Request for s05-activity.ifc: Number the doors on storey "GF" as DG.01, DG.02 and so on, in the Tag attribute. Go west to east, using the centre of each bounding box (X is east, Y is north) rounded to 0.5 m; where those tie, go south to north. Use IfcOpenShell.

First a look at what the model holds.

```python
import ifcopenshell
import ifcopenshell.util.element
import ifcopenshell.util.placement

model = ifcopenshell.open("s05-activity.ifc")
print(model.schema)
storey = next(s for s in model.by_type("IfcBuildingStorey") if s.Name == "GF")
doors = [e for e in ifcopenshell.util.element.get_decomposition(storey) if e.is_a("IfcDoor")]
for e in sorted(doors, key=lambda e: e.id()):
    origin = ifcopenshell.util.placement.get_local_placement(e.ObjectPlacement)[:3, 3]
    print(e.id(), e.Tag, e.Name, origin.round(2) + 0.0, sep=" | ")
```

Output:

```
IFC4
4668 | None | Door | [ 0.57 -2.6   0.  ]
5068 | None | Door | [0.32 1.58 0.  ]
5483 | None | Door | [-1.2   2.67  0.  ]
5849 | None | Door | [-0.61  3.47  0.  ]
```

```python
import ifcopenshell
import ifcopenshell.geom
import ifcopenshell.util.element
import ifcopenshell.util.shape

model = ifcopenshell.open("s05-activity.ifc")
settings = ifcopenshell.geom.settings()
settings.set("use-world-coords", True)


def centre(element):
    shape = ifcopenshell.geom.create_shape(settings, element)
    return ifcopenshell.util.shape.get_bbox_centroid(shape.geometry)


storey = next(s for s in model.by_type("IfcBuildingStorey") if s.Name == "GF")
doors = [e for e in ifcopenshell.util.element.get_decomposition(storey) if e.is_a("IfcDoor")]

# Insertion points can sit at a corner or the storey origin, so sort by the geometry (in metres).
centres = {e: centre(e) for e in doors}
doors.sort(key=lambda e: (round(centres[e][0] / 0.5), centres[e][1]))

for i, e in enumerate(doors, start=1):
    number = f"DG.{i:02d}"
    e.Tag = number
    print(e.id(), number)

model.write("s05-activity_rev.ifc")
```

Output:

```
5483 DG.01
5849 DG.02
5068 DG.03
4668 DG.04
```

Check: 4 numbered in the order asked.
